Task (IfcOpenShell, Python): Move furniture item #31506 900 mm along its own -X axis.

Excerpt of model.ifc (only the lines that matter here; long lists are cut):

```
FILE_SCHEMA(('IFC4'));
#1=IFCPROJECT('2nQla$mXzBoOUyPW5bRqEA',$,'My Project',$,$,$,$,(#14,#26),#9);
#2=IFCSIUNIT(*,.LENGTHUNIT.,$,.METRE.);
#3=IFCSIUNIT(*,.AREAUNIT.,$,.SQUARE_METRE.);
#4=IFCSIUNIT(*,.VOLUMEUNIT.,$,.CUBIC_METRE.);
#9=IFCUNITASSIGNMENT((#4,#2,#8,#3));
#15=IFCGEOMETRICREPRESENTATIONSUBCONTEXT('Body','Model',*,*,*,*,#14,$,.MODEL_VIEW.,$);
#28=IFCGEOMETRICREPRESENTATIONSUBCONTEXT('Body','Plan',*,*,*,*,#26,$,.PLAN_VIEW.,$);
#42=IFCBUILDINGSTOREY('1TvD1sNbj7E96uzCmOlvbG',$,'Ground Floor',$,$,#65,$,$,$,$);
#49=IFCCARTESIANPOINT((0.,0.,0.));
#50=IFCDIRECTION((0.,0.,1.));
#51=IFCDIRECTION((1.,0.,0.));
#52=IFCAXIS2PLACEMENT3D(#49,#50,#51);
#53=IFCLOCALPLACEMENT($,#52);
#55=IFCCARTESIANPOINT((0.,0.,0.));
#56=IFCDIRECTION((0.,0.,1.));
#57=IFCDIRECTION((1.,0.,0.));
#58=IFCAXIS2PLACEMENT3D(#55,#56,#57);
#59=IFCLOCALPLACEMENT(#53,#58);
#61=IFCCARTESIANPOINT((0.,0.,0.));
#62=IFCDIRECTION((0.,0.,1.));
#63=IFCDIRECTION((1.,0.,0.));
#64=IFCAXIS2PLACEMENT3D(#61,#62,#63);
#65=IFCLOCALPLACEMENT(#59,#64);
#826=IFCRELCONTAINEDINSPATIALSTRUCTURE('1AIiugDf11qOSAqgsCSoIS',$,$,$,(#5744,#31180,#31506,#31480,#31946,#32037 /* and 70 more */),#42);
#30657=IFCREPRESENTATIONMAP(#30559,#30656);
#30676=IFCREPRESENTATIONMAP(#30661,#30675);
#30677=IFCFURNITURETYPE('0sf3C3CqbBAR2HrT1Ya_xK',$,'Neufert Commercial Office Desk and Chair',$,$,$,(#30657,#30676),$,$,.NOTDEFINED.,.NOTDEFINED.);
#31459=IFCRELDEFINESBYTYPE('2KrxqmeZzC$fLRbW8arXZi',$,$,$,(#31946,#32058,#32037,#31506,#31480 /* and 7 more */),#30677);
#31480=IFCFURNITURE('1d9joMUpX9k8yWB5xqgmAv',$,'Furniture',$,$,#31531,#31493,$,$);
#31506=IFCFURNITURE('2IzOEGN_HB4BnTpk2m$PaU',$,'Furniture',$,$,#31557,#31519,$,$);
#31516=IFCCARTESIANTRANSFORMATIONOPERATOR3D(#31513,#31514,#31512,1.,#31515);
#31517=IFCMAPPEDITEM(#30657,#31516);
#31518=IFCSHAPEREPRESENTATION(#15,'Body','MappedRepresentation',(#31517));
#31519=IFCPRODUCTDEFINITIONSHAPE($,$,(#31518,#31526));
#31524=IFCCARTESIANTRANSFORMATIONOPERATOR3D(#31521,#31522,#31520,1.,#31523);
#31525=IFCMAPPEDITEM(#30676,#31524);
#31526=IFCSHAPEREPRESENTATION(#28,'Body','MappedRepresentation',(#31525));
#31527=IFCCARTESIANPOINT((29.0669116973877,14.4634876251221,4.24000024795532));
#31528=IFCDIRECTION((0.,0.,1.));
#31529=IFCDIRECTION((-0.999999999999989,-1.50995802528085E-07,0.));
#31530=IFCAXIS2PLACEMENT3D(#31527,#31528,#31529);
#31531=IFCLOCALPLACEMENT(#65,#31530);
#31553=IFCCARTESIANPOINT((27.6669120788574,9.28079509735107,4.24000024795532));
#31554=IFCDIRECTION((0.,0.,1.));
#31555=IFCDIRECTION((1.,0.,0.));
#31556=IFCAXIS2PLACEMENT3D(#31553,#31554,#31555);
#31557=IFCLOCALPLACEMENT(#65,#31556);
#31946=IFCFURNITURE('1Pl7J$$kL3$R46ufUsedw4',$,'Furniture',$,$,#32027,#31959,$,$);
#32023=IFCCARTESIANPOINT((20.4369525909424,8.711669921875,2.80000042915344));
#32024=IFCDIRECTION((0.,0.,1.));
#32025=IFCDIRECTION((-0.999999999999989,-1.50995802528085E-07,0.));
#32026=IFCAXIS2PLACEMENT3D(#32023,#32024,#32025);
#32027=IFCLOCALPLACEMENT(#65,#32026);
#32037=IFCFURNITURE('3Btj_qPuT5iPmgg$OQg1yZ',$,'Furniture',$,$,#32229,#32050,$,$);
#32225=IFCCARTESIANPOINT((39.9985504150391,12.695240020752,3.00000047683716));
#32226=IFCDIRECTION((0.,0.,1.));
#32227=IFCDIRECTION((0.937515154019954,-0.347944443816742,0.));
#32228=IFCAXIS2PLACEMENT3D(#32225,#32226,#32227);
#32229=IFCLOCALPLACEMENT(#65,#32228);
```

```python
import ifcopenshell
import ifcopenshell.api.geometry
import ifcopenshell.util.placement
import ifcopenshell.util.unit

model = ifcopenshell.open("model.ifc")
unit_scale = ifcopenshell.util.unit.calculate_unit_scale(model)

item = model.by_guid("2IzOEGN_HB4BnTpk2m$PaU")
matrix = ifcopenshell.util.placement.get_local_placement(item.ObjectPlacement)
matrix[:3, 3] -= matrix[:3, 0] * 0.9 / unit_scale
ifcopenshell.api.geometry.edit_object_placement(model, product=item, matrix=matrix, is_si=False)

print(ifcopenshell.util.placement.get_local_placement(item.ObjectPlacement).round(3) + 0.0)

model.write("model_rev.ifc")
```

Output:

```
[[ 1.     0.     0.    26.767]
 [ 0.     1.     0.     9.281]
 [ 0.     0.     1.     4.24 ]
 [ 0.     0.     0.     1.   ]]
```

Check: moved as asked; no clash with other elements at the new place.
